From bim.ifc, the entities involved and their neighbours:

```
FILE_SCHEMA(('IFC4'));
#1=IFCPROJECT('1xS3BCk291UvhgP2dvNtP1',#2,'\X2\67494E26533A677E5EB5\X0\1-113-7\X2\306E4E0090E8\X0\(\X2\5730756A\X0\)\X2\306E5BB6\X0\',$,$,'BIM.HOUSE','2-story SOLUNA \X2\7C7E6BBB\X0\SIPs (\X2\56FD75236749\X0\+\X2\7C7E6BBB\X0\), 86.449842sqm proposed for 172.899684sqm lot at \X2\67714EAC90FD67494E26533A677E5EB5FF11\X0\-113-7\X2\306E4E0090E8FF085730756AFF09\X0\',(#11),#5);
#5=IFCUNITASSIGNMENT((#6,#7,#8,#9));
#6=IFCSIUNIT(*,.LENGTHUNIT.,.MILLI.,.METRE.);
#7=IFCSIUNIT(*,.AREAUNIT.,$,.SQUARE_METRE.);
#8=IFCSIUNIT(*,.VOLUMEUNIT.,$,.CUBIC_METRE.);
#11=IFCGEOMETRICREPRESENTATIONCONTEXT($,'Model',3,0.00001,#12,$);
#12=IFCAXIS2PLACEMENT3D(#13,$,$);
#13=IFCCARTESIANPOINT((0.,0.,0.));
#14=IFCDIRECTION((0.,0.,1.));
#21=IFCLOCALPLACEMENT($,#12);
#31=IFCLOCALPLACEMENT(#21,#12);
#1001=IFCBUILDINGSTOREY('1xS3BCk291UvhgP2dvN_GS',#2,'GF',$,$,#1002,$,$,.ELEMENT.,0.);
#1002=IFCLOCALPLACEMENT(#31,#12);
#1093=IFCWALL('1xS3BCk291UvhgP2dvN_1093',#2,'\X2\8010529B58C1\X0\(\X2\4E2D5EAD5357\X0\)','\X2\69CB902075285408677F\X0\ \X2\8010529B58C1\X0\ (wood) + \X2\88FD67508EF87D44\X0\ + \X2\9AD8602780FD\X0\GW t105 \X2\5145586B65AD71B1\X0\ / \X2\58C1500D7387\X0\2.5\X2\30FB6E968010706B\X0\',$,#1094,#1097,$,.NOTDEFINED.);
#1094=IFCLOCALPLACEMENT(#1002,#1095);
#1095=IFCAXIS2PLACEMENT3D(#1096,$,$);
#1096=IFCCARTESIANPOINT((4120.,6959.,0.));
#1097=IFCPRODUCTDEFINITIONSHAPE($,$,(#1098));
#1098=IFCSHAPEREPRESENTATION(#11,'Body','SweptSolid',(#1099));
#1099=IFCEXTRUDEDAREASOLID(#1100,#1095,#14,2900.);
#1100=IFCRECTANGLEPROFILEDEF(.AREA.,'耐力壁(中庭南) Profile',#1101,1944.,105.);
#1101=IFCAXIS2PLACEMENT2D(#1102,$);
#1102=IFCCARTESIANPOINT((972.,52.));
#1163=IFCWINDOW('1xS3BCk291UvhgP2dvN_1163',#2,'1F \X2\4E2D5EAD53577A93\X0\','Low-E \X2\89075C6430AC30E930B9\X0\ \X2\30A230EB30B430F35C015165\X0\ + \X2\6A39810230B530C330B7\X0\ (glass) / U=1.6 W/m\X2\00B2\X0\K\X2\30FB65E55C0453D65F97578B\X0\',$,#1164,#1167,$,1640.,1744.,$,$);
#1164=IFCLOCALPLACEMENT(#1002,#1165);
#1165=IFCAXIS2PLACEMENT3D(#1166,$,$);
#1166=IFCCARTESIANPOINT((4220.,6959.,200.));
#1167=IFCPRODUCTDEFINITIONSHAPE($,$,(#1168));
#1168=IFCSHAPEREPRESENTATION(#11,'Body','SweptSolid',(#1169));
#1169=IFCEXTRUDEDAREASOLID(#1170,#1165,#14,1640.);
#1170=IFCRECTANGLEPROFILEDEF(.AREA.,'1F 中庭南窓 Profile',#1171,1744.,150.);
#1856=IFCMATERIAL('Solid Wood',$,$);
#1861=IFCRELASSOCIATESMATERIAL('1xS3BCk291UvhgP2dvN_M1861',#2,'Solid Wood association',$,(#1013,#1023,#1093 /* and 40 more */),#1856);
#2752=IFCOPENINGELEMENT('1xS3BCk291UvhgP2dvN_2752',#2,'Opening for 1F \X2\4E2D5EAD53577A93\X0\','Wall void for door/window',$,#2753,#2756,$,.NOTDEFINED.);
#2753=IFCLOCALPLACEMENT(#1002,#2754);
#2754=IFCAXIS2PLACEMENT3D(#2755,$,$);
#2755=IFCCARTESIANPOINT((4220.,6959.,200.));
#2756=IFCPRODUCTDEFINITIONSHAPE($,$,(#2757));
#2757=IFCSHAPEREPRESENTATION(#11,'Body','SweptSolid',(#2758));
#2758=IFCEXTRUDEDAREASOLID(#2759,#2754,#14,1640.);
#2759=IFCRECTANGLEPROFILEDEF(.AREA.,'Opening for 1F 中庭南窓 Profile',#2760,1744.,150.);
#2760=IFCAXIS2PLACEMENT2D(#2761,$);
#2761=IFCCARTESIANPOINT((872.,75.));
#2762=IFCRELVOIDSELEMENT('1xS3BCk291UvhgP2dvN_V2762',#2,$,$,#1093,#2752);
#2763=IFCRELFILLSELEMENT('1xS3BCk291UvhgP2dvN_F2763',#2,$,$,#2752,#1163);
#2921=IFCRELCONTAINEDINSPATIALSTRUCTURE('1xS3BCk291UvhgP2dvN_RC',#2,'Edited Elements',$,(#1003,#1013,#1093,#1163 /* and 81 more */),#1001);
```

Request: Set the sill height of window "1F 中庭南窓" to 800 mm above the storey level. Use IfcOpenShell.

```python
import numpy as np
import ifcopenshell
import ifcopenshell.api.geometry
import ifcopenshell.geom
import ifcopenshell.util.element
import ifcopenshell.util.placement
import ifcopenshell.util.shape
import ifcopenshell.util.unit

model = ifcopenshell.open("bim.ifc")
unit_scale = ifcopenshell.util.unit.calculate_unit_scale(model)

window = model.by_id(1163)
opening = window.FillsVoids[0].RelatingOpeningElement
storey = ifcopenshell.util.element.get_container(window, ifc_class="IfcBuildingStorey")
level = ifcopenshell.util.placement.get_local_placement(storey.ObjectPlacement)[2, 3]

# The opening's origin need not be at the sill, so measure its lowest point.
shape = ifcopenshell.geom.create_shape(ifcopenshell.geom.settings(), opening)
bottom = ifcopenshell.util.shape.get_shape_bottom_elevation(shape, shape.geometry) / unit_scale
dz = level + 0.8 / unit_scale - bottom

shift = np.array([0.0, 0.0, dz])
# The window is not placed relative to its opening, so move both.
for product in (opening, window):
    matrix = ifcopenshell.util.placement.get_local_placement(product.ObjectPlacement)
    matrix[:3, 3] += shift
    ifcopenshell.api.geometry.edit_object_placement(model, product=product, matrix=matrix, is_si=False)

print(f"moved by {dz * unit_scale:+.3f} m")

model.write("bim_v2.ifc")
```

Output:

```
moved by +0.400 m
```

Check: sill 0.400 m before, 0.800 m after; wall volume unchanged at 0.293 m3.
